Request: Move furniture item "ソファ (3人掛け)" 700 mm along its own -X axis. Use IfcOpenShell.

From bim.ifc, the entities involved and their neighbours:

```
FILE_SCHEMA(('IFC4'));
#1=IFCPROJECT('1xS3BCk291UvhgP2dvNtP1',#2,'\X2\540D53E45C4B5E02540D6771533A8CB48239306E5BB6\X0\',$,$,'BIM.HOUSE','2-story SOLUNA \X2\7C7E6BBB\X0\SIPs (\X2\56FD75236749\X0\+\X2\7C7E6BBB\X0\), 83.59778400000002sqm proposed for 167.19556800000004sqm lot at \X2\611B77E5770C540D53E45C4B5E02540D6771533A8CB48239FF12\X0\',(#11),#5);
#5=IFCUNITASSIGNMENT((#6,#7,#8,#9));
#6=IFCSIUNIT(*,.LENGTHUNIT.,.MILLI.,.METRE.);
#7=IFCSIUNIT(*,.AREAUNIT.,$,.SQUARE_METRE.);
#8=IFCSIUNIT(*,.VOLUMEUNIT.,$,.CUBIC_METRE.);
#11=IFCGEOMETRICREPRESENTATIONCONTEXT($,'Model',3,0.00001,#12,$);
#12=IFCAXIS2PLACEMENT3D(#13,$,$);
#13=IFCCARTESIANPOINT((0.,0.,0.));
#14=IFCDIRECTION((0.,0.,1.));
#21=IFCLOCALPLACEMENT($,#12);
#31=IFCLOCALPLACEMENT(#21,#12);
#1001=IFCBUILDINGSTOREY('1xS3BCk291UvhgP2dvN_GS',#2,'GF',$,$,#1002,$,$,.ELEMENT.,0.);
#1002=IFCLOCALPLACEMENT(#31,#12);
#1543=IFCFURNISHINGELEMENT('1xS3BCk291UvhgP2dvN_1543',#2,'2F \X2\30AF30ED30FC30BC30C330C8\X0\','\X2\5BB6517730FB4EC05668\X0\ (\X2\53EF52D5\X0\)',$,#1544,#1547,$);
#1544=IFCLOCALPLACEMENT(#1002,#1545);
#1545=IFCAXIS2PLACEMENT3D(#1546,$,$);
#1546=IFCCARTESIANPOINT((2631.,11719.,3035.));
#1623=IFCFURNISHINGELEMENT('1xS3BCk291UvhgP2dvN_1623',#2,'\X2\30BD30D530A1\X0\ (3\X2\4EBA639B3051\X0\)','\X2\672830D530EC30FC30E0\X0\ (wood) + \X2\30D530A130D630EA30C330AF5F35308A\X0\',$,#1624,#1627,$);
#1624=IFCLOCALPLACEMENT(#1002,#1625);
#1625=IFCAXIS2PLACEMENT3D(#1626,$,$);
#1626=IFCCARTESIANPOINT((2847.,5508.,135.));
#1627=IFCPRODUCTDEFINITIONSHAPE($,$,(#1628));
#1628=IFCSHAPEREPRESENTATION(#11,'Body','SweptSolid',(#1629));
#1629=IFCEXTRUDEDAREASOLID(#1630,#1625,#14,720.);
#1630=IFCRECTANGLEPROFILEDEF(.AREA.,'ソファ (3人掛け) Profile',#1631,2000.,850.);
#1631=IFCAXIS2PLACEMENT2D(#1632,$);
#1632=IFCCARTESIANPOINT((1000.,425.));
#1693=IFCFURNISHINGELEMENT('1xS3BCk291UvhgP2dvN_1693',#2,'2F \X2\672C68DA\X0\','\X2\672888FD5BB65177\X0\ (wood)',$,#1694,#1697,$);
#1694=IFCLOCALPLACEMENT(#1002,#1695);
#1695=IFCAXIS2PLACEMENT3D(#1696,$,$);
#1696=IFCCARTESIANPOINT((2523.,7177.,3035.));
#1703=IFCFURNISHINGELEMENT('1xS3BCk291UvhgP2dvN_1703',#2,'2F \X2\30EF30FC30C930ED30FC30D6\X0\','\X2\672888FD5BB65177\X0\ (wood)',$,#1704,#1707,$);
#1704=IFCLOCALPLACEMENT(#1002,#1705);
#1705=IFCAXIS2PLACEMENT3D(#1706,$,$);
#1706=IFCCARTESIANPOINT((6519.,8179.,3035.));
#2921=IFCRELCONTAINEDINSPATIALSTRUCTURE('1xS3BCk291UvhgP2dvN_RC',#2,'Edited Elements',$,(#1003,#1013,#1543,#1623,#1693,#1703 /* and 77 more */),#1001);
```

```python
import ifcopenshell
import ifcopenshell.api.geometry
import ifcopenshell.util.placement

model = ifcopenshell.open("bim.ifc")

item = model.by_guid("1xS3BCk291UvhgP2dvN_1623")
matrix = ifcopenshell.util.placement.get_local_placement(item.ObjectPlacement)
matrix[:3, 3] -= matrix[:3, 0] * 700.0
ifcopenshell.api.geometry.edit_object_placement(model, product=item, matrix=matrix, is_si=False)

print(ifcopenshell.util.placement.get_local_placement(item.ObjectPlacement).round(3) + 0.0)

model.write("bim-out.ifc")
```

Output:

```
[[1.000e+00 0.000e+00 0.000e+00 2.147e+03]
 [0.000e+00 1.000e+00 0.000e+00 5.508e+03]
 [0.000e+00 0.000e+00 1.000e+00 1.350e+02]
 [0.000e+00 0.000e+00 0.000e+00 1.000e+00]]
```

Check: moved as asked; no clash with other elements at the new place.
